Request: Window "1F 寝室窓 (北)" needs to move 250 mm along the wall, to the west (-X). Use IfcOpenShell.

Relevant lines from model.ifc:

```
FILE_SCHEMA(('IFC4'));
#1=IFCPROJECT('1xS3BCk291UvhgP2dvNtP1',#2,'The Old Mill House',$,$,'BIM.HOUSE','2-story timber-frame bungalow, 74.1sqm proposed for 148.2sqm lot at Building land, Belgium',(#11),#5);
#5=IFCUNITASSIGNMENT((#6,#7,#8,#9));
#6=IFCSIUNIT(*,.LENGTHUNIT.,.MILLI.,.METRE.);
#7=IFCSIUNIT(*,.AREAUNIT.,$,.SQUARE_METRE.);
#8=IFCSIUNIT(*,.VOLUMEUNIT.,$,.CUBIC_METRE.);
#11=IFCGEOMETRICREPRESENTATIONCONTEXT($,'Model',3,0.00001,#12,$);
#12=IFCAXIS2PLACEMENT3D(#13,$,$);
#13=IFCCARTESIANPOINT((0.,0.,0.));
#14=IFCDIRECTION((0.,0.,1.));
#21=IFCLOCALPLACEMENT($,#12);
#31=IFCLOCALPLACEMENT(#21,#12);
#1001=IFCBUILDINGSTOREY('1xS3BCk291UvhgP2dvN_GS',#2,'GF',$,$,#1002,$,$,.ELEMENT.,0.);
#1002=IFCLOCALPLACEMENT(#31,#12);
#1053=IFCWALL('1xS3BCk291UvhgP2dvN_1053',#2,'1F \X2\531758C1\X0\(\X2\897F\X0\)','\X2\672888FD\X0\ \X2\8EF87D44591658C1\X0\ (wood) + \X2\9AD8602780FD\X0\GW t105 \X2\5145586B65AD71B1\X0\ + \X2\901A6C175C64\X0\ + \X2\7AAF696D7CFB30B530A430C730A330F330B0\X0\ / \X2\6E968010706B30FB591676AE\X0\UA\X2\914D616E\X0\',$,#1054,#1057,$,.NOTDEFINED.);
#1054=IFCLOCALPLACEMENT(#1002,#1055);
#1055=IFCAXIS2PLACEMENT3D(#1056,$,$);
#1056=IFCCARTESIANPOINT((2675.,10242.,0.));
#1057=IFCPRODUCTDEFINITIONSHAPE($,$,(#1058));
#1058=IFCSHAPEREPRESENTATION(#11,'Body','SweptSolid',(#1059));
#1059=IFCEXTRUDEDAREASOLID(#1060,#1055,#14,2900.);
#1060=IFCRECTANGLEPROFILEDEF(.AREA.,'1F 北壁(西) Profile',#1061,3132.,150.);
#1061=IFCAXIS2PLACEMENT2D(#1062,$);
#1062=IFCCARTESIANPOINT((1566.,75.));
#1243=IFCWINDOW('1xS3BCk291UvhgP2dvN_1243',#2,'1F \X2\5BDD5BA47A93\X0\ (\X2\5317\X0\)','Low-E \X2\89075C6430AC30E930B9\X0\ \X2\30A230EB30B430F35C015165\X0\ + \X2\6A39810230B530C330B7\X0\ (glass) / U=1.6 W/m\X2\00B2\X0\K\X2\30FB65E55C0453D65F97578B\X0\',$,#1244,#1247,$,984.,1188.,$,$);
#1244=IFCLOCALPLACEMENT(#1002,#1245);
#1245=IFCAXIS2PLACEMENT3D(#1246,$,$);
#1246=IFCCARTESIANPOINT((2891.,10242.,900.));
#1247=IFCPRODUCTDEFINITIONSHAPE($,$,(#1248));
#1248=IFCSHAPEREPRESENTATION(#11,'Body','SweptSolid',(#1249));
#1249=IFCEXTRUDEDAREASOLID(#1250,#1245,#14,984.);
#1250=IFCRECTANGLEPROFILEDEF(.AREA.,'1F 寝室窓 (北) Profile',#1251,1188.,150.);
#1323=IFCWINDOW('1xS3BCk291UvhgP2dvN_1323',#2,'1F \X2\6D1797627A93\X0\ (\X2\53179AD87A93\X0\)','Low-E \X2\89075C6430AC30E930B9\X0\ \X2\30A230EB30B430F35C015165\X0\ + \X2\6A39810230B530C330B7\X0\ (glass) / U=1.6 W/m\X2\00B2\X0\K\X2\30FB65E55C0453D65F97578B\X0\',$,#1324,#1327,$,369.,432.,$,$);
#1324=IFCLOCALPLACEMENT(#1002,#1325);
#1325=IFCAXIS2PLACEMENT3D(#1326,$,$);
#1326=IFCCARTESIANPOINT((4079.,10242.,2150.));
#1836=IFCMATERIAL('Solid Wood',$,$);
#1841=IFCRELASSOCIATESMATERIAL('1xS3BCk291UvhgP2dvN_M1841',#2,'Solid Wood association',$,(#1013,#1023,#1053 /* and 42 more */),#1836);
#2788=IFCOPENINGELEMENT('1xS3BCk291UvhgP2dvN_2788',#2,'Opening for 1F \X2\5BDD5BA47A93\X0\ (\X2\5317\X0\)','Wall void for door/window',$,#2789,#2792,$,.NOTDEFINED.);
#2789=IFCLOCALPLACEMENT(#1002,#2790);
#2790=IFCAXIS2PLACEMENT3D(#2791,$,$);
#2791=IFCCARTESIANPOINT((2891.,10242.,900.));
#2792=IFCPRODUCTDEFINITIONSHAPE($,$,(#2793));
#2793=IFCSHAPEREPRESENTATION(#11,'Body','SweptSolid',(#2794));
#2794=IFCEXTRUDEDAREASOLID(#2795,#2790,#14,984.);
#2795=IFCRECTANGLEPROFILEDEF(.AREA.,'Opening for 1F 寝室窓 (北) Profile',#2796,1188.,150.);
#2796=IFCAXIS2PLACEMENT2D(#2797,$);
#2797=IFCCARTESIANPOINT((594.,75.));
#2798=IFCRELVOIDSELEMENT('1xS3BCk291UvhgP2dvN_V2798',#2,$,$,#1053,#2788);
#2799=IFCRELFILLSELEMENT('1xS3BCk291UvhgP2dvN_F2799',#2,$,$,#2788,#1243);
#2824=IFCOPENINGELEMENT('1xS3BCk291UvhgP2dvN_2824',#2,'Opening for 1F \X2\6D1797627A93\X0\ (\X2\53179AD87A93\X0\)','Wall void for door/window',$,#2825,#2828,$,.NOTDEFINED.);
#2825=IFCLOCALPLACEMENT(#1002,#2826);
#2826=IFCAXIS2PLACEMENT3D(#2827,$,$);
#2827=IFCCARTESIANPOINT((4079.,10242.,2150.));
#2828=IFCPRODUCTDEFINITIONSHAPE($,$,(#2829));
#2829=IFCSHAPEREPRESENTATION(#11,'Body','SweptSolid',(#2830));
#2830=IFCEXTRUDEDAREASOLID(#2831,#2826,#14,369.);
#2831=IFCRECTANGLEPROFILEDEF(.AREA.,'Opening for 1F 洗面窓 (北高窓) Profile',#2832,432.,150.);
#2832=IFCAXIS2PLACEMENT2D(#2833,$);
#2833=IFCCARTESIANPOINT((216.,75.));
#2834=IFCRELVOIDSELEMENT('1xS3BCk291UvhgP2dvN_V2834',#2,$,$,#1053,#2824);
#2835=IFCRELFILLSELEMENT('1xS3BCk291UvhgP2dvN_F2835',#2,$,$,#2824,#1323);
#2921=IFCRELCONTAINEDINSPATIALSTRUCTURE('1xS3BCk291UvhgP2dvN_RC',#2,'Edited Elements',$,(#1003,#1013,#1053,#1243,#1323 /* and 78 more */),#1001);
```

```python
import ifcopenshell
import ifcopenshell.api.geometry
import ifcopenshell.util.placement
import ifcopenshell.util.unit

model = ifcopenshell.open("model.ifc")
unit_scale = ifcopenshell.util.unit.calculate_unit_scale(model)

window = model.by_id(1243)
opening = window.FillsVoids[0].RelatingOpeningElement
wall = opening.VoidsElements[0].RelatingBuildingElement

wall_matrix = ifcopenshell.util.placement.get_local_placement(wall.ObjectPlacement)
shift = wall_matrix[:3, 0] * -0.25 / unit_scale
before = ifcopenshell.util.placement.get_local_placement(window.ObjectPlacement)[:3, 3].copy()

# The window is not placed relative to its opening, so move both.
for product in (opening, window):
    matrix = ifcopenshell.util.placement.get_local_placement(product.ObjectPlacement)
    matrix[:3, 3] += shift
    ifcopenshell.api.geometry.edit_object_placement(model, product=product, matrix=matrix, is_si=False)

after = ifcopenshell.util.placement.get_local_placement(window.ObjectPlacement)[:3, 3]
print("window moved by", (after - before).round(3) + 0.0)

model.write("model_edited.ifc")
```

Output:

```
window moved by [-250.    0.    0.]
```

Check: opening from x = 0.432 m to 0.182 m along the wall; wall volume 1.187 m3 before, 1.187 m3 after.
